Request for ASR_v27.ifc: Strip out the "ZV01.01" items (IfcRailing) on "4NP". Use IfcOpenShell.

First a look at what the model holds.

```python
import ifcopenshell
import ifcopenshell.util.element

model = ifcopenshell.open("ASR_v27.ifc")
print(model.schema)
storey = next(s for s in model.by_type("IfcBuildingStorey") if s.Name == "4NP")
railings = [e for e in ifcopenshell.util.element.get_decomposition(storey) if e.is_a("IfcRailing")]
seen = {}
for e in railings:
    element_type = ifcopenshell.util.element.get_type(e)
    name = element_type.Name if element_type not in (None, e) else None
    seen[name] = seen.get(name, 0) + 1
for name, count in sorted(seen.items(), key=str):
    print(count, "x", name)
```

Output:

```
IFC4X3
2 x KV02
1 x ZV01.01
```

```python
import ifcopenshell
import ifcopenshell.api.root
import ifcopenshell.util.element

model = ifcopenshell.open("ASR_v27.ifc")

storey = next(s for s in model.by_type("IfcBuildingStorey") if s.Name == "4NP")
railings = [e for e in ifcopenshell.util.element.get_decomposition(storey) if e.is_a("IfcRailing")]
targets = [e for e in railings if (t := ifcopenshell.util.element.get_type(e)) not in (None, e) and t.Name == "ZV01.01"]

for e in targets:
    ifcopenshell.api.root.remove_product(model, product=e)
print(len(targets), "removed")

model.write("ASR_v27_edited.ifc")
```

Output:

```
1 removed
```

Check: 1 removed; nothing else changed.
